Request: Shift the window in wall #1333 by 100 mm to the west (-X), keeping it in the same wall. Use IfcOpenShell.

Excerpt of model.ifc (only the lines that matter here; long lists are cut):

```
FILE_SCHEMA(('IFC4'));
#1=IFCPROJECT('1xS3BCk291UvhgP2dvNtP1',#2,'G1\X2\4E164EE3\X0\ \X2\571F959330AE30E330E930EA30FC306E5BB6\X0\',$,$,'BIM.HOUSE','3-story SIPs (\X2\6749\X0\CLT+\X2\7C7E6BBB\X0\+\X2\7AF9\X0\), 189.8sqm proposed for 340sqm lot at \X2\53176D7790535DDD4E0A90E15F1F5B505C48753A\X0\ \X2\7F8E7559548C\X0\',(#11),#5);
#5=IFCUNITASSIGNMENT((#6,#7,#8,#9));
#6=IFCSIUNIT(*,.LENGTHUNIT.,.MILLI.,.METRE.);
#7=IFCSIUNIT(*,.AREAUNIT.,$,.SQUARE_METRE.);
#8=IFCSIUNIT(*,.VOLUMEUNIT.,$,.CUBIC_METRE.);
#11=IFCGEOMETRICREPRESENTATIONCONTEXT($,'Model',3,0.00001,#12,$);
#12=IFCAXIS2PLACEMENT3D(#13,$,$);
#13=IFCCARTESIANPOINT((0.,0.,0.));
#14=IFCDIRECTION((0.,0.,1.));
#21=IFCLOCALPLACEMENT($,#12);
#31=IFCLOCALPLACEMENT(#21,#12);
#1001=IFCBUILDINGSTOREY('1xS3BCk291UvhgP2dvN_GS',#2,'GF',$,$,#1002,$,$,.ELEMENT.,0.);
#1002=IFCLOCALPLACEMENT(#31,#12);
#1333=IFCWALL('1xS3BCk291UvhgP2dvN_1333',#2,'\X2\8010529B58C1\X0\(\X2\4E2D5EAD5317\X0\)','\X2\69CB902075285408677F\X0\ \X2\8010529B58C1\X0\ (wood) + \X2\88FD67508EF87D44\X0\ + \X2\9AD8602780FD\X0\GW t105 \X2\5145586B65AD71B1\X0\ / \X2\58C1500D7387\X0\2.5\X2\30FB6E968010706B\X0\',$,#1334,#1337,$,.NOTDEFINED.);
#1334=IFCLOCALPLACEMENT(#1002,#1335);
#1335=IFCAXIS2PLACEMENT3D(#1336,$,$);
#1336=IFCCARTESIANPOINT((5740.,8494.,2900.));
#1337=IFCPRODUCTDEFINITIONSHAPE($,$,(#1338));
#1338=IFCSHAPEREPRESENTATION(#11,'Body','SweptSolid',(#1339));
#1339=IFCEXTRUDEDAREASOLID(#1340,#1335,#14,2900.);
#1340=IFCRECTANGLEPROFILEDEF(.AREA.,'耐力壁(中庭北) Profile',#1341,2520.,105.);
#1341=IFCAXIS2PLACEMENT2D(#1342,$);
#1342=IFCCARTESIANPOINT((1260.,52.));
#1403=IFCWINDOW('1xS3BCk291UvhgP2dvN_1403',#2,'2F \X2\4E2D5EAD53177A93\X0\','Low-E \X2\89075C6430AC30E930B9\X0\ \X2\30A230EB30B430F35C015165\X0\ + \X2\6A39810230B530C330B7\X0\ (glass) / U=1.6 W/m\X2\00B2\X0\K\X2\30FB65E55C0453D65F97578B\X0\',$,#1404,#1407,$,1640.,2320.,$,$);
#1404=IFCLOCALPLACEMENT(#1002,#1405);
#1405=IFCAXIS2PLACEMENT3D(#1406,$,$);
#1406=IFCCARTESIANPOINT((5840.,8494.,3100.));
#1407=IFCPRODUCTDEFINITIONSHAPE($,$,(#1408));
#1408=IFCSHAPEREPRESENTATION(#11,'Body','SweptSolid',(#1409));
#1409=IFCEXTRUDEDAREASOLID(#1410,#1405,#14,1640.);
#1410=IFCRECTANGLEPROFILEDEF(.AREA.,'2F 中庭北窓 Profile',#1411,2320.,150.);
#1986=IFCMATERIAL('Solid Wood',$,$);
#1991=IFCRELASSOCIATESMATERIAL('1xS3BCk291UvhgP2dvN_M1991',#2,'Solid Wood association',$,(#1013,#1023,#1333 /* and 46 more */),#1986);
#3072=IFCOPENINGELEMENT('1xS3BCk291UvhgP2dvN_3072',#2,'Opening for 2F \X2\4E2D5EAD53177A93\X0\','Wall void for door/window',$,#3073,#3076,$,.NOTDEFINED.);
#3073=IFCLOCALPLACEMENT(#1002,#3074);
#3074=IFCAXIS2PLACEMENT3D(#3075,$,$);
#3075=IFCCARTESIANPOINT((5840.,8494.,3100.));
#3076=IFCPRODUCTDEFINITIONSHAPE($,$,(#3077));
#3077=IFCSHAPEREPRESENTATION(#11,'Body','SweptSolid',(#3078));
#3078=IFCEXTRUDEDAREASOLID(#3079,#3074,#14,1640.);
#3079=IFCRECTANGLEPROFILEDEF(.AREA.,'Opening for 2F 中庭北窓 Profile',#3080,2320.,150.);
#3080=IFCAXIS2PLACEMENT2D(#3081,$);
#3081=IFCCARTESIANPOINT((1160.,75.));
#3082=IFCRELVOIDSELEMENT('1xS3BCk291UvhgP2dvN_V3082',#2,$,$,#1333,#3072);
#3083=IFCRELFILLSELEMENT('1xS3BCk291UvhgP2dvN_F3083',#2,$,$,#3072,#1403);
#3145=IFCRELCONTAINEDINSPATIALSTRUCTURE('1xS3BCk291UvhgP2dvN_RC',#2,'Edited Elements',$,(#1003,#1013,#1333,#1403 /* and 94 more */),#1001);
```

```python
import ifcopenshell
import ifcopenshell.api.geometry
import ifcopenshell.util.placement
import ifcopenshell.util.unit

model = ifcopenshell.open("model.ifc")
unit_scale = ifcopenshell.util.unit.calculate_unit_scale(model)

window = model.by_guid("1xS3BCk291UvhgP2dvN_1403")
opening = window.FillsVoids[0].RelatingOpeningElement
wall = opening.VoidsElements[0].RelatingBuildingElement

wall_matrix = ifcopenshell.util.placement.get_local_placement(wall.ObjectPlacement)
shift = wall_matrix[:3, 0] * -0.1 / unit_scale
before = ifcopenshell.util.placement.get_local_placement(window.ObjectPlacement)[:3, 3].copy()

# The window is not placed relative to its opening, so move both.
for product in (opening, window):
    matrix = ifcopenshell.util.placement.get_local_placement(product.ObjectPlacement)
    matrix[:3, 3] += shift
    ifcopenshell.api.geometry.edit_object_placement(model, product=product, matrix=matrix, is_si=False)

after = ifcopenshell.util.placement.get_local_placement(window.ObjectPlacement)[:3, 3]
print("window moved by", (after - before).round(3) + 0.0)

model.write("model_updated.ifc")
```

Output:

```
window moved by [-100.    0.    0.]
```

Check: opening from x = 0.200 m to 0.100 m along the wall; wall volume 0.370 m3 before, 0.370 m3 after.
